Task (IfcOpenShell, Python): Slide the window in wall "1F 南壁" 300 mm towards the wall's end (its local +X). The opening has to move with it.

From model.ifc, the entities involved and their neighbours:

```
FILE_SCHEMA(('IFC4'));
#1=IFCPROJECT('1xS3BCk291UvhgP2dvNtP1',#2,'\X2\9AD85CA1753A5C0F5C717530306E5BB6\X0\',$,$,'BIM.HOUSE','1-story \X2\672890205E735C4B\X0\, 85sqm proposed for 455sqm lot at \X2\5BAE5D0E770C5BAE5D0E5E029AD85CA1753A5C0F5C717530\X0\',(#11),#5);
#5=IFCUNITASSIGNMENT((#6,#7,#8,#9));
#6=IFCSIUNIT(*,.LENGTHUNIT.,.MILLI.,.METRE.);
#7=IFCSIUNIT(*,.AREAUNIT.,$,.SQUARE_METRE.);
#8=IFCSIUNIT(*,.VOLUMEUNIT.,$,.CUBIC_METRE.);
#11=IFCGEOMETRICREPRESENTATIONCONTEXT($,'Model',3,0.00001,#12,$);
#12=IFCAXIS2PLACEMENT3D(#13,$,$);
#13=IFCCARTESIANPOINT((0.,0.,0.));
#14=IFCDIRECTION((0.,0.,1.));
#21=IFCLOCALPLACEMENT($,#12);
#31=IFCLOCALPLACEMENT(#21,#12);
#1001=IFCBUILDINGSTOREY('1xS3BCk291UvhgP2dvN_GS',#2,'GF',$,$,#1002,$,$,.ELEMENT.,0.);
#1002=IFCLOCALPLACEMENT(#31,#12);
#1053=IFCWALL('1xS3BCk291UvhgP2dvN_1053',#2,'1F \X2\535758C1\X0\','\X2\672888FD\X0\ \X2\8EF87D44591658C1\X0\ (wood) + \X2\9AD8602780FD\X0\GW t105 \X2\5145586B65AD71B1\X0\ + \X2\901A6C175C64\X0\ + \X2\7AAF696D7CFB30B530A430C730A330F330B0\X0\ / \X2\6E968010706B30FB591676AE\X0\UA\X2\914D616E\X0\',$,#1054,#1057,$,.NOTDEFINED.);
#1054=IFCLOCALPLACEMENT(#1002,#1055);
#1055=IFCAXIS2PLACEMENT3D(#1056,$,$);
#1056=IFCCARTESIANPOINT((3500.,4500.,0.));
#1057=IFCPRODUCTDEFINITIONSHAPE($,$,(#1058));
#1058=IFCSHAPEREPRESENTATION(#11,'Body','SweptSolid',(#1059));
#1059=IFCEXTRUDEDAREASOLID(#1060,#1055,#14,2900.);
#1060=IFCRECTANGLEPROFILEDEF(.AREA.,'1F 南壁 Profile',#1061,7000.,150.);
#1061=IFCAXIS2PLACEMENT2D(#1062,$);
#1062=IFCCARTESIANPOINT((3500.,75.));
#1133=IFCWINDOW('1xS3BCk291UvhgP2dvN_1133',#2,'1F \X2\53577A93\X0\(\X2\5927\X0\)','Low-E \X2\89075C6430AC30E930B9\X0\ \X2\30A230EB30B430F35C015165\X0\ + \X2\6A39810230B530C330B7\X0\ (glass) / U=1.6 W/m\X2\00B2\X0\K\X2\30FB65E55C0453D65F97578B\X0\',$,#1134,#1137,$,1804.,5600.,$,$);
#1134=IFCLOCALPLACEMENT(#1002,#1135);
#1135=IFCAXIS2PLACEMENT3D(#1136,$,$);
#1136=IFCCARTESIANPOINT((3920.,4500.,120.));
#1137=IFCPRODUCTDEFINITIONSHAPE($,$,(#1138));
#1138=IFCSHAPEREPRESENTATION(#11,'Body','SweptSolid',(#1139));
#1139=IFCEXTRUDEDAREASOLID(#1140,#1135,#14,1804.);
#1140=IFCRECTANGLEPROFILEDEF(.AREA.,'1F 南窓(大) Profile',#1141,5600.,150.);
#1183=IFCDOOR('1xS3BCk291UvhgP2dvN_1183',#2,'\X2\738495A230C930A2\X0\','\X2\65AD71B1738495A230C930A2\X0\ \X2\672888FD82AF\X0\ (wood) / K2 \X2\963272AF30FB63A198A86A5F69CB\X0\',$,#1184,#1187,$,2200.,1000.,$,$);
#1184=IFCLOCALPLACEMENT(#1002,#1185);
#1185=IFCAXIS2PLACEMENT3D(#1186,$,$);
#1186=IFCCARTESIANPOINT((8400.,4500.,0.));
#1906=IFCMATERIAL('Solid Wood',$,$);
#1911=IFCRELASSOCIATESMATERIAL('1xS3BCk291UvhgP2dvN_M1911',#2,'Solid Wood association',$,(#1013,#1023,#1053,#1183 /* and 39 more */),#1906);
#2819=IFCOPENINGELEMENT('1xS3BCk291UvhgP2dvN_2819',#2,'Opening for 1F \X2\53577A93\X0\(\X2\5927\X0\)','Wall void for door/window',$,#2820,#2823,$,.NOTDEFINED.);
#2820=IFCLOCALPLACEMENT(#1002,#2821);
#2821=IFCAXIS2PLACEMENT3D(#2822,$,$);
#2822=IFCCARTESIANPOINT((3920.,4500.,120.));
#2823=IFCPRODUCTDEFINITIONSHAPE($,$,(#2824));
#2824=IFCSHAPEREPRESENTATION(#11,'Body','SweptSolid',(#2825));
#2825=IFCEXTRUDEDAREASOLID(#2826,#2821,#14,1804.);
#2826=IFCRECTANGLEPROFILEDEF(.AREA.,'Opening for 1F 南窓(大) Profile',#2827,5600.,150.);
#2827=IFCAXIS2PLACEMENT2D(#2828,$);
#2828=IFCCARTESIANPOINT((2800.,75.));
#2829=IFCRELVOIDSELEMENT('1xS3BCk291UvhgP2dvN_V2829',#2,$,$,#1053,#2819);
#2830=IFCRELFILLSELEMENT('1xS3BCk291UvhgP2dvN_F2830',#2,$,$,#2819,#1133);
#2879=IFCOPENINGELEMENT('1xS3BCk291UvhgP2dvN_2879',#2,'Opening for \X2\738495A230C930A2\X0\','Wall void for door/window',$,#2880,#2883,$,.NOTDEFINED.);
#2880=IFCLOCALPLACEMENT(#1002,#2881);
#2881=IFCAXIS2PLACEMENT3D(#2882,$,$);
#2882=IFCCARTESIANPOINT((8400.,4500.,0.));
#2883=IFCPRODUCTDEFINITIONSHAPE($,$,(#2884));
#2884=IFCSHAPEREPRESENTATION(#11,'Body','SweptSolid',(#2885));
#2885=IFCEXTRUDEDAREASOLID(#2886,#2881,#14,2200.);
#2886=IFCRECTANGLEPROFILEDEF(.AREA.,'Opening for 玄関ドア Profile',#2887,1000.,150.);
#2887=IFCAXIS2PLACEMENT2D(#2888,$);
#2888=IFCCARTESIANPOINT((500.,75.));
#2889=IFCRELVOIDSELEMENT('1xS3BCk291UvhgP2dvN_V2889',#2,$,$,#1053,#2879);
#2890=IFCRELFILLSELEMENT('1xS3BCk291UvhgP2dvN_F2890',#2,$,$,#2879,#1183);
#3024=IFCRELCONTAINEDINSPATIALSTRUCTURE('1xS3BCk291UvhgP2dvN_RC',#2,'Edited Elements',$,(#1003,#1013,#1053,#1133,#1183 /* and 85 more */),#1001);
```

```python
import ifcopenshell
import ifcopenshell.api.geometry
import ifcopenshell.util.placement
import ifcopenshell.util.unit

model = ifcopenshell.open("model.ifc")
unit_scale = ifcopenshell.util.unit.calculate_unit_scale(model)

window = model.by_guid("1xS3BCk291UvhgP2dvN_1133")
opening = window.FillsVoids[0].RelatingOpeningElement
wall = opening.VoidsElements[0].RelatingBuildingElement

wall_matrix = ifcopenshell.util.placement.get_local_placement(wall.ObjectPlacement)
shift = wall_matrix[:3, 0] * 0.3 / unit_scale
before = ifcopenshell.util.placement.get_local_placement(window.ObjectPlacement)[:3, 3].copy()

# The window is not placed relative to its opening, so move both.
for product in (opening, window):
    matrix = ifcopenshell.util.placement.get_local_placement(product.ObjectPlacement)
    matrix[:3, 3] += shift
    ifcopenshell.api.geometry.edit_object_placement(model, product=product, matrix=matrix, is_si=False)

after = ifcopenshell.util.placement.get_local_placement(window.ObjectPlacement)[:3, 3]
print("window moved by", (after - before).round(3) + 0.0)

model.write("model-out.ifc")
```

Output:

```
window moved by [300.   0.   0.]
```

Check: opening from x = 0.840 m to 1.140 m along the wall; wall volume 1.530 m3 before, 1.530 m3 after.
